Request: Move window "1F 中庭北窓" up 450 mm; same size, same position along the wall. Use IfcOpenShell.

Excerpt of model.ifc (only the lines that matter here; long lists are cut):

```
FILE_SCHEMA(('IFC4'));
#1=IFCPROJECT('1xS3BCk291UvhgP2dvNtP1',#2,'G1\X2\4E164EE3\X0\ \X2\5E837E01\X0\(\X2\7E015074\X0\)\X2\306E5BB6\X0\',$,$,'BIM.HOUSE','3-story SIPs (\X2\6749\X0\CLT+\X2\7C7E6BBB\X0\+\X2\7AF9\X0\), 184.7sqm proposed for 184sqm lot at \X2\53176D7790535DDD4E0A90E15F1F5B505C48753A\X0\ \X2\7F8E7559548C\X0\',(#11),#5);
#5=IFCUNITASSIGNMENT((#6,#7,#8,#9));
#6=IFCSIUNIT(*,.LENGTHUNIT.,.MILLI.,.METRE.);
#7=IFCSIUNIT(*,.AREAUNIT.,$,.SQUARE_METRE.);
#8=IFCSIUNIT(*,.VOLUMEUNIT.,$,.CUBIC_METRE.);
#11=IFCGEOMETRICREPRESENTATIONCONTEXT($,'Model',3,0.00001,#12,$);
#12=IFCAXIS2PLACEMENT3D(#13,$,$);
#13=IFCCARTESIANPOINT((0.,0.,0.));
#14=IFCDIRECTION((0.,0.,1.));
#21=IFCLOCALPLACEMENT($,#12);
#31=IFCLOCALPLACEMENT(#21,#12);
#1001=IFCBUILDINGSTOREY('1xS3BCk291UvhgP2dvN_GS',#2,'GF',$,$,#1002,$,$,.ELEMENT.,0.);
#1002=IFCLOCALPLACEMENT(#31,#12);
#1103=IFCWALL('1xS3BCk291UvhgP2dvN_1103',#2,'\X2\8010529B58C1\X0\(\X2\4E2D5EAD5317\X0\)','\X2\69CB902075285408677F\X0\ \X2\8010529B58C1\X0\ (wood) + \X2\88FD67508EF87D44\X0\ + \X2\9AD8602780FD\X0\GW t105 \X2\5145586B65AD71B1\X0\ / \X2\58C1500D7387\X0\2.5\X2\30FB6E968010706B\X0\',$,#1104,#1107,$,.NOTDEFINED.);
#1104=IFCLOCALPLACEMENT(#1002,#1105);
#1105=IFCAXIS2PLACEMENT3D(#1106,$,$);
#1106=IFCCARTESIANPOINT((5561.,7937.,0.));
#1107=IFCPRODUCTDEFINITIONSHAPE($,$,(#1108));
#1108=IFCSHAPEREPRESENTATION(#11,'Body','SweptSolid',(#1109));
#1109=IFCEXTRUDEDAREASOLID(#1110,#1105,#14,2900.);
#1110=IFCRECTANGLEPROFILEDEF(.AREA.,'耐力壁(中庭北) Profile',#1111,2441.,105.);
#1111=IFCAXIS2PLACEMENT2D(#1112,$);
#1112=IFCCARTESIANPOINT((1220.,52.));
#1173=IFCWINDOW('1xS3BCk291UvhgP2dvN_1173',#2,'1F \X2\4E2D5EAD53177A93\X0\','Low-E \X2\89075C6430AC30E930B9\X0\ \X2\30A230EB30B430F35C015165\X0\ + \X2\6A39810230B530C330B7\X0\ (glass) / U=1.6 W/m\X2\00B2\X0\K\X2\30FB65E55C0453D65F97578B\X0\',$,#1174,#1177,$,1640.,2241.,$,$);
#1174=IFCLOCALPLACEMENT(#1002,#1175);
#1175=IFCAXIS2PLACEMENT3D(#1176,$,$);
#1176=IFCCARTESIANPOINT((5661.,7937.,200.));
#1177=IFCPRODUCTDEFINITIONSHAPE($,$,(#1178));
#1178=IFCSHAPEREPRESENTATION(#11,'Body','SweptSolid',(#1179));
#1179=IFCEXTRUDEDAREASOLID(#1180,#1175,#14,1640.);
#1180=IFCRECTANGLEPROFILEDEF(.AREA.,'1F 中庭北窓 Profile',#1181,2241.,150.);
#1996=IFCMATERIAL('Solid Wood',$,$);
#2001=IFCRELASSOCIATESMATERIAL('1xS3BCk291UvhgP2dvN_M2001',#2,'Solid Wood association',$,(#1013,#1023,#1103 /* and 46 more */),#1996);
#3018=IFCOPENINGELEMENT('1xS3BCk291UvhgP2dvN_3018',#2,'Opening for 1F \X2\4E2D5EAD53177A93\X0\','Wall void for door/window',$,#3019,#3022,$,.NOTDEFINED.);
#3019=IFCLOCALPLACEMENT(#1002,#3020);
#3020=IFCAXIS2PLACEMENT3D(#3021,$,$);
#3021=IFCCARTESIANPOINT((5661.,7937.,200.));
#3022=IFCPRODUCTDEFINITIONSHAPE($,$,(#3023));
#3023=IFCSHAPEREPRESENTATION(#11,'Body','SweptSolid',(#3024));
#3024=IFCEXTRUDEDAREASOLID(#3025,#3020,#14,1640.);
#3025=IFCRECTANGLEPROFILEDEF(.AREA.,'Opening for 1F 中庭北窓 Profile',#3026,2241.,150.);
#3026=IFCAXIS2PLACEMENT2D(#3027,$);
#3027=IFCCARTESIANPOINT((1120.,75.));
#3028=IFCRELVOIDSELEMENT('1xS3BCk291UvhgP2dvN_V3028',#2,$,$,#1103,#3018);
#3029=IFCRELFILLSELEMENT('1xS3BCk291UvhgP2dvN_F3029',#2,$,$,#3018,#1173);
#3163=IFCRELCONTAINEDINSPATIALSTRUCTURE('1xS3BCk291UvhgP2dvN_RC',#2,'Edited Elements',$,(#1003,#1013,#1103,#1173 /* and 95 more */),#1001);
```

```python
import numpy as np
import ifcopenshell
import ifcopenshell.api.geometry
import ifcopenshell.util.placement
import ifcopenshell.util.unit

model = ifcopenshell.open("model.ifc")
unit_scale = ifcopenshell.util.unit.calculate_unit_scale(model)

window = model.by_id(1173)
opening = window.FillsVoids[0].RelatingOpeningElement
dz = 0.45 / unit_scale

shift = np.array([0.0, 0.0, dz])
# The window is not placed relative to its opening, so move both.
for product in (opening, window):
    matrix = ifcopenshell.util.placement.get_local_placement(product.ObjectPlacement)
    matrix[:3, 3] += shift
    ifcopenshell.api.geometry.edit_object_placement(model, product=product, matrix=matrix, is_si=False)

print(f"moved by {dz * unit_scale:+.3f} m")

model.write("model_edited.ifc")
```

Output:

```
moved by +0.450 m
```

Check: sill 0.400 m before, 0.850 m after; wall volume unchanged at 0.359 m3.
